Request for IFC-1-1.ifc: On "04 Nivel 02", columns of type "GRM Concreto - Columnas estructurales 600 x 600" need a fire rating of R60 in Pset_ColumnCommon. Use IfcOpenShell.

First a look at what the model holds.

```python
import ifcopenshell
import ifcopenshell.util.element

model = ifcopenshell.open("IFC-1-1.ifc")
print(model.schema)
storey = next(s for s in model.by_type("IfcBuildingStorey") if s.Name == "04 Nivel 02")
columns = [e for e in ifcopenshell.util.element.get_decomposition(storey) if e.is_a("IfcColumn")]
seen = {}
for e in columns:
    element_type = ifcopenshell.util.element.get_type(e)
    key = (element_type.Name if element_type != e and element_type else None, ifcopenshell.util.element.get_pset(e, "Pset_ColumnCommon", "FireRating"))
    seen[key] = seen.get(key, 0) + 1
for (name, value), count in sorted(seen.items(), key=str):
    print(count, "x", name, "|", value)
```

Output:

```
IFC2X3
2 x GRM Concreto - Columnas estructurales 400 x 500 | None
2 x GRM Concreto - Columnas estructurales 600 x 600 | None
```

```python
import ifcopenshell
import ifcopenshell.api.pset
import ifcopenshell.util.element

model = ifcopenshell.open("IFC-1-1.ifc")

storey = next(s for s in model.by_type("IfcBuildingStorey") if s.Name == "04 Nivel 02")
columns = [e for e in ifcopenshell.util.element.get_decomposition(storey) if e.is_a("IfcColumn")]

count = 0
for e in columns:
    element_type = ifcopenshell.util.element.get_type(e)
    if element_type in (None, e) or element_type.Name != "GRM Concreto - Columnas estructurales 600 x 600":
        continue
    # add_pset returns the element's existing set when there is one.
    pset = ifcopenshell.api.pset.add_pset(model, product=e, name="Pset_ColumnCommon")
    ifcopenshell.api.pset.edit_pset(model, pset=pset, properties={"FireRating": "R60"})
    count += 1

print(count, "columns updated")

model.write("IFC-1-1-out.ifc")
```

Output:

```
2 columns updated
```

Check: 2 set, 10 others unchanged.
